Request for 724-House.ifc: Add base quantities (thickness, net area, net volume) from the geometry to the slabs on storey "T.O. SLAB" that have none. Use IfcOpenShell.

First a look at what the model holds.

```python
import ifcopenshell
import ifcopenshell.util.element
import ifcopenshell.util.unit

model = ifcopenshell.open("724-House.ifc")
print(model.schema)
for unit_type in ("LENGTHUNIT", "AREAUNIT", "VOLUMEUNIT"):
    print(unit_type, ifcopenshell.util.unit.calculate_unit_scale(model, unit_type))
storey = next(s for s in model.by_type("IfcBuildingStorey") if s.Name == "T.O. SLAB")
slabs = [e for e in ifcopenshell.util.element.get_decomposition(storey) if e.is_a("IfcSlab")]
for e in sorted(slabs, key=lambda e: e.id()):
    print(e.id(), e.is_a(), e.Name, list(ifcopenshell.util.element.get_psets(e, qtos_only=True)), sep=" | ")
```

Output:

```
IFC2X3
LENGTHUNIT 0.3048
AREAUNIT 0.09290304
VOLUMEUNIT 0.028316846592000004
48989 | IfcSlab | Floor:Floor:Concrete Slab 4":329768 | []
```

```python
import ifcopenshell
import ifcopenshell.api.pset
import ifcopenshell.geom
import ifcopenshell.util.element
import ifcopenshell.util.shape
import ifcopenshell.util.unit

model = ifcopenshell.open("724-House.ifc")
unit_scale = ifcopenshell.util.unit.calculate_unit_scale(model)
area_scale = ifcopenshell.util.unit.calculate_unit_scale(model, "AREAUNIT")
volume_scale = ifcopenshell.util.unit.calculate_unit_scale(model, "VOLUMEUNIT")
settings = ifcopenshell.geom.settings()

storey = next(s for s in model.by_type("IfcBuildingStorey") if s.Name == "T.O. SLAB")
slabs = [e for e in ifcopenshell.util.element.get_decomposition(storey) if e.is_a("IfcSlab")]

for e in sorted(slabs, key=lambda e: e.id()):
    if ifcopenshell.util.element.get_psets(e, qtos_only=True, should_inherit=False):
        continue
    # Geometry comes back in metres, in the element's own axes.
    shape = ifcopenshell.geom.create_shape(settings, e)
    values = {
        "Width": ifcopenshell.util.shape.get_z(shape.geometry) / unit_scale,
        "NetArea": ifcopenshell.util.shape.get_footprint_area(shape.geometry) / area_scale,
        "NetVolume": ifcopenshell.util.shape.get_volume(shape.geometry) / volume_scale,
    }
    qto = ifcopenshell.api.pset.add_qto(model, product=e, name="BaseQuantities")
    ifcopenshell.api.pset.edit_qto(model, qto=qto, properties=values)
    print(e.id(), {k: round(v, 3) for k, v in values.items()})

model.write("724-House_v2.ifc")
```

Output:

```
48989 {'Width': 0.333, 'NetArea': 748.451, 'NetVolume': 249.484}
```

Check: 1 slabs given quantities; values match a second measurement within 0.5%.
